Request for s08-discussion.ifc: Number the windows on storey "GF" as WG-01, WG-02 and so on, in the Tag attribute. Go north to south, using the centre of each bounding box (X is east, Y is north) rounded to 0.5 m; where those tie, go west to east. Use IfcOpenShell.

First a look at what the model holds.

```python
import ifcopenshell
import ifcopenshell.util.element
import ifcopenshell.util.placement

model = ifcopenshell.open("s08-discussion.ifc")
print(model.schema)
storey = next(s for s in model.by_type("IfcBuildingStorey") if s.Name == "GF")
windows = [e for e in ifcopenshell.util.element.get_decomposition(storey) if e.is_a("IfcWindow")]
for e in sorted(windows, key=lambda e: e.id()):
    origin = ifcopenshell.util.placement.get_local_placement(e.ObjectPlacement)[:3, 3]
    print(e.id(), e.Tag, e.Name, origin.round(2) + 0.0, sep=" | ")
```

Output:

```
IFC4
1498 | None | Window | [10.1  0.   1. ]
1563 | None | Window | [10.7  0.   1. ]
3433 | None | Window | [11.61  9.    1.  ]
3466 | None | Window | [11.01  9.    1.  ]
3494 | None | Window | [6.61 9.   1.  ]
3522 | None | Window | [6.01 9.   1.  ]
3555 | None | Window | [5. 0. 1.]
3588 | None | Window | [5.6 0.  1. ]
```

```python
import ifcopenshell
import ifcopenshell.geom
import ifcopenshell.util.element
import ifcopenshell.util.shape

model = ifcopenshell.open("s08-discussion.ifc")
settings = ifcopenshell.geom.settings()
settings.set("use-world-coords", True)


def centre(element):
    shape = ifcopenshell.geom.create_shape(settings, element)
    return ifcopenshell.util.shape.get_bbox_centroid(shape.geometry)


storey = next(s for s in model.by_type("IfcBuildingStorey") if s.Name == "GF")
windows = [e for e in ifcopenshell.util.element.get_decomposition(storey) if e.is_a("IfcWindow")]

# Insertion points can sit at a corner or the storey origin, so sort by the geometry (in metres).
centres = {e: centre(e) for e in windows}
windows.sort(key=lambda e: (-round(centres[e][1] / 0.5), centres[e][0]))

for i, e in enumerate(windows, start=1):
    number = f"WG-{i:02d}"
    e.Tag = number
    print(e.id(), number)

model.write("s08-discussion_updated.ifc")
```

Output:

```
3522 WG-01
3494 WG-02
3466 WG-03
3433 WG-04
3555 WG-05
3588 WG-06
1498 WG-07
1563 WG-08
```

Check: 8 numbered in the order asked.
